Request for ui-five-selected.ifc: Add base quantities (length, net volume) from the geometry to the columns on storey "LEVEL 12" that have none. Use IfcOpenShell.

First a look at what the model holds.

```python
import ifcopenshell
import ifcopenshell.util.element
import ifcopenshell.util.unit

model = ifcopenshell.open("ui-five-selected.ifc")
print(model.schema)
for unit_type in ("LENGTHUNIT", "AREAUNIT", "VOLUMEUNIT"):
    print(unit_type, ifcopenshell.util.unit.calculate_unit_scale(model, unit_type))
storey = next(s for s in model.by_type("IfcBuildingStorey") if s.Name == "LEVEL 12")
columns = [e for e in ifcopenshell.util.element.get_decomposition(storey) if e.is_a("IfcColumn")]
for e in sorted(columns, key=lambda e: e.id()):
    print(e.id(), e.is_a(), e.Name, list(ifcopenshell.util.element.get_psets(e, qtos_only=True)), sep=" | ")
```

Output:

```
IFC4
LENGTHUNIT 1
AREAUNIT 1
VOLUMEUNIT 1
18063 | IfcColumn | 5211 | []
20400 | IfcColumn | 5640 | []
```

```python
import ifcopenshell
import ifcopenshell.api.pset
import ifcopenshell.geom
import ifcopenshell.util.element
import ifcopenshell.util.shape
import ifcopenshell.util.unit

model = ifcopenshell.open("ui-five-selected.ifc")
unit_scale = ifcopenshell.util.unit.calculate_unit_scale(model)
volume_scale = ifcopenshell.util.unit.calculate_unit_scale(model, "VOLUMEUNIT")
settings = ifcopenshell.geom.settings()

storey = next(s for s in model.by_type("IfcBuildingStorey") if s.Name == "LEVEL 12")
columns = [e for e in ifcopenshell.util.element.get_decomposition(storey) if e.is_a("IfcColumn")]

for e in sorted(columns, key=lambda e: e.id()):
    if ifcopenshell.util.element.get_psets(e, qtos_only=True, should_inherit=False):
        continue
    # Geometry comes back in metres, in the element's own axes.
    shape = ifcopenshell.geom.create_shape(settings, e)
    values = {
        "Length": ifcopenshell.util.shape.get_z(shape.geometry) / unit_scale,
        "NetVolume": ifcopenshell.util.shape.get_volume(shape.geometry) / volume_scale,
    }
    qto = ifcopenshell.api.pset.add_qto(model, product=e, name="Qto_ColumnBaseQuantities")
    ifcopenshell.api.pset.edit_qto(model, qto=qto, properties=values)
    print(e.id(), {k: round(v, 3) for k, v in values.items()})

model.write("ui-five-selected_v2.ifc")
```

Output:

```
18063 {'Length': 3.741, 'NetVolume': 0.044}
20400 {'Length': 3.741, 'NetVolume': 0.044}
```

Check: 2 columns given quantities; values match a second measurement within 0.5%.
